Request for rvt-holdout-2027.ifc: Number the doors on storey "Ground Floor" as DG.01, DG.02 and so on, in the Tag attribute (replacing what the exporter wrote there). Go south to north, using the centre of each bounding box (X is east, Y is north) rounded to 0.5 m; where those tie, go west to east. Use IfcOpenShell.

First a look at what the model holds.

```python
import ifcopenshell
import ifcopenshell.util.element
import ifcopenshell.util.placement

model = ifcopenshell.open("rvt-holdout-2027.ifc")
print(model.schema)
storey = next(s for s in model.by_type("IfcBuildingStorey") if s.Name == "Ground Floor")
doors = [e for e in ifcopenshell.util.element.get_decomposition(storey) if e.is_a("IfcDoor")]
for e in sorted(doors, key=lambda e: e.id()):
    origin = ifcopenshell.util.placement.get_local_placement(e.ObjectPlacement)[:3, 3]
    print(e.id(), e.Tag, e.Name, origin.round(2) + 0.0, sep=" | ")
```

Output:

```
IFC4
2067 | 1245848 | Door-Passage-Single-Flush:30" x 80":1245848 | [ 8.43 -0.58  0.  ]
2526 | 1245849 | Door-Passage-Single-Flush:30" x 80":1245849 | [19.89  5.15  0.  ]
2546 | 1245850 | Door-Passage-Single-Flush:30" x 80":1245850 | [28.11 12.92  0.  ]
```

```python
import ifcopenshell
import ifcopenshell.geom
import ifcopenshell.util.element
import ifcopenshell.util.shape

model = ifcopenshell.open("rvt-holdout-2027.ifc")
settings = ifcopenshell.geom.settings()
settings.set("use-world-coords", True)


def centre(element):
    shape = ifcopenshell.geom.create_shape(settings, element)
    return ifcopenshell.util.shape.get_bbox_centroid(shape.geometry)


storey = next(s for s in model.by_type("IfcBuildingStorey") if s.Name == "Ground Floor")
doors = [e for e in ifcopenshell.util.element.get_decomposition(storey) if e.is_a("IfcDoor")]

# Insertion points can sit at a corner or the storey origin, so sort by the geometry (in metres).
centres = {e: centre(e) for e in doors}
doors.sort(key=lambda e: (round(centres[e][1] / 0.5), centres[e][0]))

for i, e in enumerate(doors, start=1):
    number = f"DG.{i:02d}"
    e.Tag = number
    print(e.id(), number)

model.write("rvt-holdout-2027_updated.ifc")
```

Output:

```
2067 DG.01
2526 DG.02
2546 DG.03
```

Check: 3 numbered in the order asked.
